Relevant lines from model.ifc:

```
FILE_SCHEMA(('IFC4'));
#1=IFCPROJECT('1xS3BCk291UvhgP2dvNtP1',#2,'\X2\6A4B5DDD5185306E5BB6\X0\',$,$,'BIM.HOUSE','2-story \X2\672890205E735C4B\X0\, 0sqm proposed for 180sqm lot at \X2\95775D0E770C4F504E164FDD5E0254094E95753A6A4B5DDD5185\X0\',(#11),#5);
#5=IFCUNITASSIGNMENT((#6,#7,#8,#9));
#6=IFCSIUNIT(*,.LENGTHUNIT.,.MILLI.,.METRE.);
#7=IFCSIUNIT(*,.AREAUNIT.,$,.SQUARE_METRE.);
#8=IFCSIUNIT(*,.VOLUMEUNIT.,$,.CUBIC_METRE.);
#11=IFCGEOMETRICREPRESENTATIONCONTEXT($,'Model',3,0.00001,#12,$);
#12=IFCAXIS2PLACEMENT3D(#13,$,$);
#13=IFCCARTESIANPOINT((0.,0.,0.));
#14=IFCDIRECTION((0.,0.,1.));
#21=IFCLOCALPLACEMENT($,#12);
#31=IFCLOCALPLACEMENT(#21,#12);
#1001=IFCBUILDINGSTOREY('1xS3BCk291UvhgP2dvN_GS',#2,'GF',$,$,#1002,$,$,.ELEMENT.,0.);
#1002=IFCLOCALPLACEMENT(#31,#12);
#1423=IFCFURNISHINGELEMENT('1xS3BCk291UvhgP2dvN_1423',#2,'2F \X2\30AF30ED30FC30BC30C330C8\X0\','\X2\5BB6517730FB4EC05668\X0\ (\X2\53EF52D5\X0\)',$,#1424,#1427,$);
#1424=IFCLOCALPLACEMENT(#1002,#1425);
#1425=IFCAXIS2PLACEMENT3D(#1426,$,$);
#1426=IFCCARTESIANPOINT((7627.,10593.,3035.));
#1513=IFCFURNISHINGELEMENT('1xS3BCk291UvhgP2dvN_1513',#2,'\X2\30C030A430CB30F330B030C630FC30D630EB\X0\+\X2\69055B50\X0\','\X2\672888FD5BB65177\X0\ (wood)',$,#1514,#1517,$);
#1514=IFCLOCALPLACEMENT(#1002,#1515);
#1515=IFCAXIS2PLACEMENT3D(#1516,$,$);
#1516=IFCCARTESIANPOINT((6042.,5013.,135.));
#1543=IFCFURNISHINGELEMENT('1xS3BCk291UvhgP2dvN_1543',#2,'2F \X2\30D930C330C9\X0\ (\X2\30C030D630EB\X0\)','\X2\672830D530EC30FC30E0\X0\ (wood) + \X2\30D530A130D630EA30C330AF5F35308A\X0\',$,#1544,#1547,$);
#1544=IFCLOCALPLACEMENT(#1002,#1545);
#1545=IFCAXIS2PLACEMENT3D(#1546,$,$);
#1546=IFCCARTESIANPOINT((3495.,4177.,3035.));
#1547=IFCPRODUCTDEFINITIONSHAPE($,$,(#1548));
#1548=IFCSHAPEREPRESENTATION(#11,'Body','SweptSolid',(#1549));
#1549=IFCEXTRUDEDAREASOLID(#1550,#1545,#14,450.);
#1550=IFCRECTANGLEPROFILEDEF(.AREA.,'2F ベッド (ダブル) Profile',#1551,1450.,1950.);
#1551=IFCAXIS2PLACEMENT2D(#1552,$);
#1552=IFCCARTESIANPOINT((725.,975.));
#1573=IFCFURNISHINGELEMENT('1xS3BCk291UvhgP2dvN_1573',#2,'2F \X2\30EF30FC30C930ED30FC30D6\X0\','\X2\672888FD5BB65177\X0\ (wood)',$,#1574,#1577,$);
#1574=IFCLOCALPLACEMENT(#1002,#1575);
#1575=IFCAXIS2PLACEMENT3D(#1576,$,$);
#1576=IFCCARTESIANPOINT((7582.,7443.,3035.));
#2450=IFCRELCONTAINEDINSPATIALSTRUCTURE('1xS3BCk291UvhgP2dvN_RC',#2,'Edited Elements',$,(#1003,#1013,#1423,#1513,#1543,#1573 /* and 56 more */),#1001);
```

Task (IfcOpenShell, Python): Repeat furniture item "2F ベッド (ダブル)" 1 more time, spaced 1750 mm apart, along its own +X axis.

```python
import ifcopenshell
import ifcopenshell.api.geometry
import ifcopenshell.api.root
import ifcopenshell.util.element
import ifcopenshell.util.placement

model = ifcopenshell.open("model.ifc")


def reuse_history(source, copy):
    """copy_class also copies each property set's owner history, people and application; keep the originals."""
    for rel in copy.IsDefinedBy:
        if rel.is_a("IfcRelDefinesByProperties") and (history := rel.RelatingPropertyDefinition.OwnerHistory):
            rel.RelatingPropertyDefinition.OwnerHistory = source.OwnerHistory
            ifcopenshell.util.element.remove_deep2(model, history)


source = model.by_guid("1xS3BCk291UvhgP2dvN_1543")
base = ifcopenshell.util.placement.get_local_placement(source.ObjectPlacement)
step = base[:3, 0] * 1750.0

for i in range(1, 2):
    copy = ifcopenshell.api.root.copy_class(model, product=source)
    copy.Representation = ifcopenshell.util.element.copy_deep(
        model, source.Representation, exclude=["IfcGeometricRepresentationContext", "IfcRepresentationMap"]
    )
    reuse_history(source, copy)
    matrix = base.copy()
    matrix[:3, 3] += i * step
    print("added at", matrix[:3, 3].round(3) + 0.0)
    ifcopenshell.api.geometry.edit_object_placement(model, product=copy, matrix=matrix, is_si=False)

model.write("model_edited.ifc")
```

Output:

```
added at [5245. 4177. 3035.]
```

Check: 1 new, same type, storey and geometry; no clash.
